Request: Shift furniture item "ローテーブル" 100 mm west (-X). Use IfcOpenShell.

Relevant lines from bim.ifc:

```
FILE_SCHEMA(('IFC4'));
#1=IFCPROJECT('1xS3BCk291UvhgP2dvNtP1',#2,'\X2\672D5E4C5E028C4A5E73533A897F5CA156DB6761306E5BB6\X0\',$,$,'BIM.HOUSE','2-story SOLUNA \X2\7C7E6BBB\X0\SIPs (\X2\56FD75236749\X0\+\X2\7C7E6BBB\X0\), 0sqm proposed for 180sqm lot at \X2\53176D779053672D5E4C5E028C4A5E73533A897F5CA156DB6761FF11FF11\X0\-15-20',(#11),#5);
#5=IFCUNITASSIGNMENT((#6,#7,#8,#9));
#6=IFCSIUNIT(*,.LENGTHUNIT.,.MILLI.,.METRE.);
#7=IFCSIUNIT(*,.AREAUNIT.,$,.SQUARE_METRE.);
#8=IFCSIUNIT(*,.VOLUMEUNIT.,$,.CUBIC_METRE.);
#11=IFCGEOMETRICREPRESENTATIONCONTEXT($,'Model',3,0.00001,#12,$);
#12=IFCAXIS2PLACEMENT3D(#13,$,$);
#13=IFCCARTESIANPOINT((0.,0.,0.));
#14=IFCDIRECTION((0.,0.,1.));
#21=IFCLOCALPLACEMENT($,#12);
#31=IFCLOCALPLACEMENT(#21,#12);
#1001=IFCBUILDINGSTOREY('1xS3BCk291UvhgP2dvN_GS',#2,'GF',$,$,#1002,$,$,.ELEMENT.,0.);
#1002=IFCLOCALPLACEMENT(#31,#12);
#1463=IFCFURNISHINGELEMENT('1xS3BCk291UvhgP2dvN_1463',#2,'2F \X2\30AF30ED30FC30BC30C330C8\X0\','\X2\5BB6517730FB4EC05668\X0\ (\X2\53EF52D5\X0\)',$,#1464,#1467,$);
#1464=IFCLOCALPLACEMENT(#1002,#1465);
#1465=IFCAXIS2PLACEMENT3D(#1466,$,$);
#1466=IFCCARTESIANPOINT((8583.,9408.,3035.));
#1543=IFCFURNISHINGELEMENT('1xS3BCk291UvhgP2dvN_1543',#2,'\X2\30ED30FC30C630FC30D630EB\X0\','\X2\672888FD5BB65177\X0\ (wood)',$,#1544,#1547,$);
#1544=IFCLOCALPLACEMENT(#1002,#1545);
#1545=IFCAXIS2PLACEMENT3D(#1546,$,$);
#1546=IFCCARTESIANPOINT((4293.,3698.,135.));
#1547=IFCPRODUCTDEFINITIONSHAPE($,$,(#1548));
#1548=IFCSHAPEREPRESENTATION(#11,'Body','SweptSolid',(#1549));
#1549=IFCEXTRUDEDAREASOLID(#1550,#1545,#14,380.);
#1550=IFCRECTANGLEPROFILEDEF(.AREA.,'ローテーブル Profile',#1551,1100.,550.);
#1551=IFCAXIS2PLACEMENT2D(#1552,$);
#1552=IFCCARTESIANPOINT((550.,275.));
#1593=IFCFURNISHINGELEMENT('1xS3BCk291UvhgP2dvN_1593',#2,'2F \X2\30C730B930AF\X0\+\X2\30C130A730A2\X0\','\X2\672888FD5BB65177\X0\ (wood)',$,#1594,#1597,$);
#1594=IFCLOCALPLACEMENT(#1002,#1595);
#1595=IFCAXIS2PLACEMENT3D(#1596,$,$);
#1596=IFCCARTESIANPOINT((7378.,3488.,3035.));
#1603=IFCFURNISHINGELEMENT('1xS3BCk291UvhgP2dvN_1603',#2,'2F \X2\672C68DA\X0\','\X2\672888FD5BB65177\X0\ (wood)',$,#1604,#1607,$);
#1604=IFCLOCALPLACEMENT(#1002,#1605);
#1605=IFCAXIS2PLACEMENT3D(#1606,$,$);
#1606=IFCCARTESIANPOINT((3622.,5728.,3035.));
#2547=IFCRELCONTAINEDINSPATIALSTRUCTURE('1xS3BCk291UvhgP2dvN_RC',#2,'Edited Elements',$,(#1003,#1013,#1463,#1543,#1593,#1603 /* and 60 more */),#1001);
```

```python
import ifcopenshell
import ifcopenshell.api.geometry
import ifcopenshell.util.placement
import ifcopenshell.util.unit

model = ifcopenshell.open("bim.ifc")
unit_scale = ifcopenshell.util.unit.calculate_unit_scale(model)

item = model.by_id(1543)
matrix = ifcopenshell.util.placement.get_local_placement(item.ObjectPlacement)
matrix[0, 3] -= 0.1 / unit_scale
ifcopenshell.api.geometry.edit_object_placement(model, product=item, matrix=matrix, is_si=False)

print(ifcopenshell.util.placement.get_local_placement(item.ObjectPlacement).round(3) + 0.0)

model.write("bim_updated.ifc")
```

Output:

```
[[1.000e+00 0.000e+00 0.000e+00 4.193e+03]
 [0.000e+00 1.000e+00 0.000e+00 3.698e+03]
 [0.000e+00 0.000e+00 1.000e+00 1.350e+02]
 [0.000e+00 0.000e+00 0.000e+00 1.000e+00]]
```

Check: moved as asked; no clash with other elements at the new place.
